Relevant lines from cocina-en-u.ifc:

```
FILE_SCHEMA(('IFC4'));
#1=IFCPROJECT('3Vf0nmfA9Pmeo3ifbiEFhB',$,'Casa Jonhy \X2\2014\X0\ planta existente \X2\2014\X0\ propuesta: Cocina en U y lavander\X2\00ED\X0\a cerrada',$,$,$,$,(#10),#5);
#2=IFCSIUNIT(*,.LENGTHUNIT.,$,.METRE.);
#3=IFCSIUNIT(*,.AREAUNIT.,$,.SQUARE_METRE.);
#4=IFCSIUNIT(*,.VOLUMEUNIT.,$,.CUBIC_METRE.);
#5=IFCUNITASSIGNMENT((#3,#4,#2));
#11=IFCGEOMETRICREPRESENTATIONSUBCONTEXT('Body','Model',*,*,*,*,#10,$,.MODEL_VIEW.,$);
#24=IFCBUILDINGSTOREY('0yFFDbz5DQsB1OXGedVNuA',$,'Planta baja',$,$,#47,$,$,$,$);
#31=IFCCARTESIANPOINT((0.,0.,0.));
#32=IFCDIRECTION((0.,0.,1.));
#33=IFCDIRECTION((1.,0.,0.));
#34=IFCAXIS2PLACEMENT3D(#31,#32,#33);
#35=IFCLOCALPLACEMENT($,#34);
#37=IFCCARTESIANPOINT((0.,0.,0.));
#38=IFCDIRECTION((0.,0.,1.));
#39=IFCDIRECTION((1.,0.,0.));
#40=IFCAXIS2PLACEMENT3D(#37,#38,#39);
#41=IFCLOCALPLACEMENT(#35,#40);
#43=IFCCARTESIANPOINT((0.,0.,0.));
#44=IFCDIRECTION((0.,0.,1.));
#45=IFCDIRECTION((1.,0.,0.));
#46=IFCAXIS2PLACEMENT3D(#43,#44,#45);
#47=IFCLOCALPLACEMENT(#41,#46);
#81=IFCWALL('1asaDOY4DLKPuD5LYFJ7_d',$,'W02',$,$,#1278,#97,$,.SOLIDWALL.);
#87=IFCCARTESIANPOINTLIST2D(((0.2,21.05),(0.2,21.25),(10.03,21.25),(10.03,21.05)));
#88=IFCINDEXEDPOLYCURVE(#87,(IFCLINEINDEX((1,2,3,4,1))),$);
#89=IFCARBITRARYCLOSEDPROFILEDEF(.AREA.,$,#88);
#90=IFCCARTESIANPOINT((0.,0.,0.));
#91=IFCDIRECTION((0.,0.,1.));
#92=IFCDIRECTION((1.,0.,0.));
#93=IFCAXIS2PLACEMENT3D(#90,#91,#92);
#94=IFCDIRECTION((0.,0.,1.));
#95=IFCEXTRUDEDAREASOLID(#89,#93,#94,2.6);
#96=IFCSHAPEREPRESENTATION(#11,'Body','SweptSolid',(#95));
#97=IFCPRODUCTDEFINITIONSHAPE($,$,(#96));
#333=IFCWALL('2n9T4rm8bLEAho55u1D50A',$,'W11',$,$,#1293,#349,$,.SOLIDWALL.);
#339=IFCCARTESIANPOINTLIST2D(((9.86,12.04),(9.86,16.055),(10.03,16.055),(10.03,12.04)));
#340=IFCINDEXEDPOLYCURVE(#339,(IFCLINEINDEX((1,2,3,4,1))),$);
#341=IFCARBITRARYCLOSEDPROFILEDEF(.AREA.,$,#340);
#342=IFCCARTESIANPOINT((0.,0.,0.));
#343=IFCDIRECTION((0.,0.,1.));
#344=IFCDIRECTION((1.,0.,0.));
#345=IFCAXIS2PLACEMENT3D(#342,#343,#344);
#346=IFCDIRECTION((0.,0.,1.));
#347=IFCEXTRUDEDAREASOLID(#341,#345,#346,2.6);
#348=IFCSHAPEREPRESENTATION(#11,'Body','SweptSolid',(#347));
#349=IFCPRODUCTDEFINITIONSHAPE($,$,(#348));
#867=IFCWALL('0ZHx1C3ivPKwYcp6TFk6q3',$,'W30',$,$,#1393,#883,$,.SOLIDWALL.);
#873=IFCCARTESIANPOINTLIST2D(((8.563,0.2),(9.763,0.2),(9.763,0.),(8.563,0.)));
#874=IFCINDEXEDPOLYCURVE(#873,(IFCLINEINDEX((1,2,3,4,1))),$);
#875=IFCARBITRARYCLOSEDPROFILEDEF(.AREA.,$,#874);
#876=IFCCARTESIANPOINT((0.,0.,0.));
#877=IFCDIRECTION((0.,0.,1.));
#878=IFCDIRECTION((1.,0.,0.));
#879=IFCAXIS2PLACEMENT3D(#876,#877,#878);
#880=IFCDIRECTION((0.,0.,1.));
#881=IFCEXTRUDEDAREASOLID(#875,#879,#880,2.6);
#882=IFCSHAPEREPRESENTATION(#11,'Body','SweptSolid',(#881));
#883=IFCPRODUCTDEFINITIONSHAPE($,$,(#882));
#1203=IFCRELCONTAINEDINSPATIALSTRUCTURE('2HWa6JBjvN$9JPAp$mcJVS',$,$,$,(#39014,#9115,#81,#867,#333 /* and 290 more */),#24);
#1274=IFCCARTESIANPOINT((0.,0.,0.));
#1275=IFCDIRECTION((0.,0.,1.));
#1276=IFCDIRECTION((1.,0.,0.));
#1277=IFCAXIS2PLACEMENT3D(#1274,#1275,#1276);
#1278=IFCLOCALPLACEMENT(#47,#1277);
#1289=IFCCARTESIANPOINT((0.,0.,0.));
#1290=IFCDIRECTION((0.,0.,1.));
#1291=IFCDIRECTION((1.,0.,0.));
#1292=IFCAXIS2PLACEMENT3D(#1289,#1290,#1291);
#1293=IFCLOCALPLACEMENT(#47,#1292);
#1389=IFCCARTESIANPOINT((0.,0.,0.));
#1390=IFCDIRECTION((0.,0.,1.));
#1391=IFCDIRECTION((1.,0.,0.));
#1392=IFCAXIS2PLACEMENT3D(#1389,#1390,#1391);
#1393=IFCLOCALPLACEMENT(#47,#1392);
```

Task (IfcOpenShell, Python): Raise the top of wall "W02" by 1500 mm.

```python
import ifcopenshell
import ifcopenshell.geom
import ifcopenshell.util.representation
import ifcopenshell.util.shape
import ifcopenshell.util.unit

model = ifcopenshell.open("cocina-en-u.ifc")
unit_scale = ifcopenshell.util.unit.calculate_unit_scale(model)
settings = ifcopenshell.geom.settings()


def volume(element):
    """Net volume in cubic metres, openings subtracted."""
    shape = ifcopenshell.geom.create_shape(settings, element)
    return ifcopenshell.util.shape.get_volume(shape.geometry)


wall = model.by_id(81)
before = volume(wall)

body = ifcopenshell.util.representation.get_representation(wall, "Model", "Body")
solid = body.Items[0]
old_height = solid.Depth
solid.Depth += 1.5 / unit_scale
after = volume(wall)

print(f"height {old_height:g} -> {solid.Depth:g}, volume {before:.3f} -> {after:.3f} m3")

model.write("cocina-en-u_edited.ifc")
```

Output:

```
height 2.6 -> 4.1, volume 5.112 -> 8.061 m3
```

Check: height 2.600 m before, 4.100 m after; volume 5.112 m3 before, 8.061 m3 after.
